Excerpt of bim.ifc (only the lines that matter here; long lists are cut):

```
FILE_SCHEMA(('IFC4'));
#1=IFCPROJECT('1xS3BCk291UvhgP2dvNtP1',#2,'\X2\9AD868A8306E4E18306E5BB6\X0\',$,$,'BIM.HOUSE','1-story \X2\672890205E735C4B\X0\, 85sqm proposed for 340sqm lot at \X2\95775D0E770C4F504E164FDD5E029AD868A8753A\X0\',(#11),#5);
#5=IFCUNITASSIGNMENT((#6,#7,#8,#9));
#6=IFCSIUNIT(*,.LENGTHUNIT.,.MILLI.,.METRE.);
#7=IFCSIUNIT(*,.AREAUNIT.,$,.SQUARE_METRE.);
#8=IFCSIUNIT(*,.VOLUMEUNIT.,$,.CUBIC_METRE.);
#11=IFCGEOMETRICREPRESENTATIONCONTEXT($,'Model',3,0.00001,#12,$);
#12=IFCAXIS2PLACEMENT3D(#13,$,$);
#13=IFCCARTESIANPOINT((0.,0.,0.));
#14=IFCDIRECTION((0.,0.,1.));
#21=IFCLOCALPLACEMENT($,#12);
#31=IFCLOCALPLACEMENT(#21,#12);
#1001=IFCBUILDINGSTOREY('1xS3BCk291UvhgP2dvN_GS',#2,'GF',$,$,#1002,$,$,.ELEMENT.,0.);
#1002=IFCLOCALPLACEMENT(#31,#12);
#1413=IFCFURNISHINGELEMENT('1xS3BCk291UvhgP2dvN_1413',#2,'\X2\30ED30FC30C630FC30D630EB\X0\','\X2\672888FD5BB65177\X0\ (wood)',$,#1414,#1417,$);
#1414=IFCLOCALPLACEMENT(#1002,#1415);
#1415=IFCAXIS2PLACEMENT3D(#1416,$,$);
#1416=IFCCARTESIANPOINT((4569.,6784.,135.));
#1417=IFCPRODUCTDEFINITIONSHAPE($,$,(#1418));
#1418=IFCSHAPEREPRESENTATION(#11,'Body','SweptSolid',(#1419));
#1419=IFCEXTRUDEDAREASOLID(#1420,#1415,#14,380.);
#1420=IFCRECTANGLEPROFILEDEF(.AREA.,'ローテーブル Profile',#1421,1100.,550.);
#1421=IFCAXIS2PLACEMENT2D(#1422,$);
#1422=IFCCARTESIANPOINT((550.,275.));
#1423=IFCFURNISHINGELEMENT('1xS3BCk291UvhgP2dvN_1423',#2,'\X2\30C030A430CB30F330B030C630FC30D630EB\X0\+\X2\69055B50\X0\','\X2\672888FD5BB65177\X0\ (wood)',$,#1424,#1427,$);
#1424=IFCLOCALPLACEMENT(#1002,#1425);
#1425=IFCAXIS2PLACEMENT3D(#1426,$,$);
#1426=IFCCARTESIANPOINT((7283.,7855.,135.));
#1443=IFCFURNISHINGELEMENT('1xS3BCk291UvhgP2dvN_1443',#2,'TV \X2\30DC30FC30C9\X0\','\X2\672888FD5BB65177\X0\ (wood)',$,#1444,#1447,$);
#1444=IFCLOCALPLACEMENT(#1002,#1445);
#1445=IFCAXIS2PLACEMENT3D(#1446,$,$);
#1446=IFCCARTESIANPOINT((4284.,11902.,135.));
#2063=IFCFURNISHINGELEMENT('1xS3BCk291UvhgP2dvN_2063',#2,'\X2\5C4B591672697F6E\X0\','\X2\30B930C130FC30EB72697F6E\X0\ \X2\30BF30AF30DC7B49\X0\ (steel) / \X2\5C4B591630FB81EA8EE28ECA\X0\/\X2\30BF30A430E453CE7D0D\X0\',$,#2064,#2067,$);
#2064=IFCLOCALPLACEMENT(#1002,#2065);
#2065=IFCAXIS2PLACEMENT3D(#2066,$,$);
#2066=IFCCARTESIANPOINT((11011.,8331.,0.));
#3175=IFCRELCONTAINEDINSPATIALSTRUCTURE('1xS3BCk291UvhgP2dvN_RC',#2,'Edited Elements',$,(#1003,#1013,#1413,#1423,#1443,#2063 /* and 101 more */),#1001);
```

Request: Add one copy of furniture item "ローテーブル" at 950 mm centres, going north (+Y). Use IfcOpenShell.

```python
import numpy as np
import ifcopenshell
import ifcopenshell.api.geometry
import ifcopenshell.api.root
import ifcopenshell.util.element
import ifcopenshell.util.placement

model = ifcopenshell.open("bim.ifc")


def reuse_history(source, copy):
    """copy_class also copies each property set's owner history, people and application; keep the originals."""
    for rel in copy.IsDefinedBy:
        if rel.is_a("IfcRelDefinesByProperties") and (history := rel.RelatingPropertyDefinition.OwnerHistory):
            rel.RelatingPropertyDefinition.OwnerHistory = source.OwnerHistory
            ifcopenshell.util.element.remove_deep2(model, history)


source = model.by_guid("1xS3BCk291UvhgP2dvN_1413")
base = ifcopenshell.util.placement.get_local_placement(source.ObjectPlacement)
step = np.array([0.0, 1.0, 0.0]) * 950.0

for i in range(1, 2):
    copy = ifcopenshell.api.root.copy_class(model, product=source)
    copy.Representation = ifcopenshell.util.element.copy_deep(
        model, source.Representation, exclude=["IfcGeometricRepresentationContext", "IfcRepresentationMap"]
    )
    reuse_history(source, copy)
    matrix = base.copy()
    matrix[:3, 3] += i * step
    print("added at", matrix[:3, 3].round(3) + 0.0)
    ifcopenshell.api.geometry.edit_object_placement(model, product=copy, matrix=matrix, is_si=False)

model.write("bim-out.ifc")
```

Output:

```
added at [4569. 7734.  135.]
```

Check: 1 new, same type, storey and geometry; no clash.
